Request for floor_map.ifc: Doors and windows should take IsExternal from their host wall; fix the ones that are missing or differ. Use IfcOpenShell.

First a look at what the model holds.

```python
import ifcopenshell
import ifcopenshell.util.element

model = ifcopenshell.open("floor_map.ifc")
print(model.schema)
seen = {}
for e in model.by_type("IfcDoor") + model.by_type("IfcWindow"):
    if not e.FillsVoids:
        continue
    host = e.FillsVoids[0].RelatingOpeningElement.VoidsElements[0].RelatingBuildingElement
    own = ifcopenshell.util.element.get_pset(e, f"Pset_{e.is_a()[3:].removesuffix('StandardCase')}Common", "IsExternal")
    wall = ifcopenshell.util.element.get_pset(host, "Pset_WallCommon", "IsExternal")
    seen[e.is_a(), own, wall] = seen.get((e.is_a(), own, wall), 0) + 1
for (cls, own, wall), count in sorted(seen.items(), key=str):
    print(count, cls, "IsExternal:", own, "| host wall:", wall)
```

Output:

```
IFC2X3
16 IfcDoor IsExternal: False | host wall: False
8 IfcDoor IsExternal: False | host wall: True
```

```python
import ifcopenshell
import ifcopenshell.api.pset
import ifcopenshell.util.element

model = ifcopenshell.open("floor_map.ifc")

count = 0
for ifc_class, pset_name in (("IfcDoor", "Pset_DoorCommon"), ("IfcWindow", "Pset_WindowCommon")):
    for e in model.by_type(ifc_class):
        if not e.FillsVoids:
            continue
        host = e.FillsVoids[0].RelatingOpeningElement.VoidsElements[0].RelatingBuildingElement
        external = ifcopenshell.util.element.get_pset(host, "Pset_WallCommon", "IsExternal")
        if external is None or ifcopenshell.util.element.get_pset(e, pset_name, "IsExternal") == external:
            continue
        pset = ifcopenshell.api.pset.add_pset(model, product=e, name=pset_name)
        ifcopenshell.api.pset.edit_pset(model, pset=pset, properties={"IsExternal": external})
        count += 1

print(count, "updated")

model.write("floor_map_rev.ifc")
```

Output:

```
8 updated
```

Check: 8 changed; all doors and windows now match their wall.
